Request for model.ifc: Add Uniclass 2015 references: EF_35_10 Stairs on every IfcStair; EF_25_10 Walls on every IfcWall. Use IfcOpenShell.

First a look at what the model holds.

```python
import ifcopenshell

model = ifcopenshell.open("model.ifc")
print(model.schema)
print("classifications:", [c.Name for c in model.by_type("IfcClassification")])
for ifc_class in ("IfcDoor", "IfcRoof", "IfcStair", "IfcWall", "IfcWindow"):
    print(ifc_class, len(model.by_type(ifc_class)))
```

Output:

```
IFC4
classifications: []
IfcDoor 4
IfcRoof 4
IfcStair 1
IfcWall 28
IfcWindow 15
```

```python
import ifcopenshell
import ifcopenshell.api.classification

model = ifcopenshell.open("model.ifc")

system = ifcopenshell.api.classification.add_classification(model, classification="Uniclass 2015")

codes = {
    "IfcStair": ("EF_35_10", "Stairs"),
    "IfcWall": ("EF_25_10", "Walls"),
}
for ifc_class, (code, name) in codes.items():
    products = model.by_type(ifc_class)
    ifcopenshell.api.classification.add_reference(
        model, products=products, classification=system, identification=code, name=name
    )
    print(code, len(products))

model.write("model_v2.ifc")
```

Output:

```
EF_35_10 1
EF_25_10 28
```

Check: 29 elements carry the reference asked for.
